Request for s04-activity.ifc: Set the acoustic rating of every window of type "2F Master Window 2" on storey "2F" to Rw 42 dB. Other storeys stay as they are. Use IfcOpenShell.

First a look at what the model holds.

```python
import ifcopenshell
import ifcopenshell.util.element

model = ifcopenshell.open("s04-activity.ifc")
print(model.schema)
storey = next(s for s in model.by_type("IfcBuildingStorey") if s.Name == "2F")
windows = [e for e in ifcopenshell.util.element.get_decomposition(storey) if e.is_a("IfcWindow")]
seen = {}
for e in windows:
    element_type = ifcopenshell.util.element.get_type(e)
    key = (element_type.Name if element_type != e and element_type else None, ifcopenshell.util.element.get_pset(e, "Pset_WindowCommon", "AcousticRating"))
    seen[key] = seen.get(key, 0) + 1
for (name, value), count in sorted(seen.items(), key=str):
    print(count, "x", name, "|", value)
```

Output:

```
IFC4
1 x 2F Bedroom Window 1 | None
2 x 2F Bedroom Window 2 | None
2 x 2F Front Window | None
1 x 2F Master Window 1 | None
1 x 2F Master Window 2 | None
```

```python
import ifcopenshell
import ifcopenshell.api.pset
import ifcopenshell.util.element

model = ifcopenshell.open("s04-activity.ifc")

storey = next(s for s in model.by_type("IfcBuildingStorey") if s.Name == "2F")
windows = [e for e in ifcopenshell.util.element.get_decomposition(storey) if e.is_a("IfcWindow")]

count = 0
for e in windows:
    element_type = ifcopenshell.util.element.get_type(e)
    if element_type in (None, e) or element_type.Name != "2F Master Window 2":
        continue
    # add_pset returns the element's existing set when there is one.
    pset = ifcopenshell.api.pset.add_pset(model, product=e, name="Pset_WindowCommon")
    ifcopenshell.api.pset.edit_pset(model, pset=pset, properties={"AcousticRating": "Rw 42 dB"})
    count += 1

print(count, "windows updated")

model.write("s04-activity_rev.ifc")
```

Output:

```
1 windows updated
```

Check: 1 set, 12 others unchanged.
